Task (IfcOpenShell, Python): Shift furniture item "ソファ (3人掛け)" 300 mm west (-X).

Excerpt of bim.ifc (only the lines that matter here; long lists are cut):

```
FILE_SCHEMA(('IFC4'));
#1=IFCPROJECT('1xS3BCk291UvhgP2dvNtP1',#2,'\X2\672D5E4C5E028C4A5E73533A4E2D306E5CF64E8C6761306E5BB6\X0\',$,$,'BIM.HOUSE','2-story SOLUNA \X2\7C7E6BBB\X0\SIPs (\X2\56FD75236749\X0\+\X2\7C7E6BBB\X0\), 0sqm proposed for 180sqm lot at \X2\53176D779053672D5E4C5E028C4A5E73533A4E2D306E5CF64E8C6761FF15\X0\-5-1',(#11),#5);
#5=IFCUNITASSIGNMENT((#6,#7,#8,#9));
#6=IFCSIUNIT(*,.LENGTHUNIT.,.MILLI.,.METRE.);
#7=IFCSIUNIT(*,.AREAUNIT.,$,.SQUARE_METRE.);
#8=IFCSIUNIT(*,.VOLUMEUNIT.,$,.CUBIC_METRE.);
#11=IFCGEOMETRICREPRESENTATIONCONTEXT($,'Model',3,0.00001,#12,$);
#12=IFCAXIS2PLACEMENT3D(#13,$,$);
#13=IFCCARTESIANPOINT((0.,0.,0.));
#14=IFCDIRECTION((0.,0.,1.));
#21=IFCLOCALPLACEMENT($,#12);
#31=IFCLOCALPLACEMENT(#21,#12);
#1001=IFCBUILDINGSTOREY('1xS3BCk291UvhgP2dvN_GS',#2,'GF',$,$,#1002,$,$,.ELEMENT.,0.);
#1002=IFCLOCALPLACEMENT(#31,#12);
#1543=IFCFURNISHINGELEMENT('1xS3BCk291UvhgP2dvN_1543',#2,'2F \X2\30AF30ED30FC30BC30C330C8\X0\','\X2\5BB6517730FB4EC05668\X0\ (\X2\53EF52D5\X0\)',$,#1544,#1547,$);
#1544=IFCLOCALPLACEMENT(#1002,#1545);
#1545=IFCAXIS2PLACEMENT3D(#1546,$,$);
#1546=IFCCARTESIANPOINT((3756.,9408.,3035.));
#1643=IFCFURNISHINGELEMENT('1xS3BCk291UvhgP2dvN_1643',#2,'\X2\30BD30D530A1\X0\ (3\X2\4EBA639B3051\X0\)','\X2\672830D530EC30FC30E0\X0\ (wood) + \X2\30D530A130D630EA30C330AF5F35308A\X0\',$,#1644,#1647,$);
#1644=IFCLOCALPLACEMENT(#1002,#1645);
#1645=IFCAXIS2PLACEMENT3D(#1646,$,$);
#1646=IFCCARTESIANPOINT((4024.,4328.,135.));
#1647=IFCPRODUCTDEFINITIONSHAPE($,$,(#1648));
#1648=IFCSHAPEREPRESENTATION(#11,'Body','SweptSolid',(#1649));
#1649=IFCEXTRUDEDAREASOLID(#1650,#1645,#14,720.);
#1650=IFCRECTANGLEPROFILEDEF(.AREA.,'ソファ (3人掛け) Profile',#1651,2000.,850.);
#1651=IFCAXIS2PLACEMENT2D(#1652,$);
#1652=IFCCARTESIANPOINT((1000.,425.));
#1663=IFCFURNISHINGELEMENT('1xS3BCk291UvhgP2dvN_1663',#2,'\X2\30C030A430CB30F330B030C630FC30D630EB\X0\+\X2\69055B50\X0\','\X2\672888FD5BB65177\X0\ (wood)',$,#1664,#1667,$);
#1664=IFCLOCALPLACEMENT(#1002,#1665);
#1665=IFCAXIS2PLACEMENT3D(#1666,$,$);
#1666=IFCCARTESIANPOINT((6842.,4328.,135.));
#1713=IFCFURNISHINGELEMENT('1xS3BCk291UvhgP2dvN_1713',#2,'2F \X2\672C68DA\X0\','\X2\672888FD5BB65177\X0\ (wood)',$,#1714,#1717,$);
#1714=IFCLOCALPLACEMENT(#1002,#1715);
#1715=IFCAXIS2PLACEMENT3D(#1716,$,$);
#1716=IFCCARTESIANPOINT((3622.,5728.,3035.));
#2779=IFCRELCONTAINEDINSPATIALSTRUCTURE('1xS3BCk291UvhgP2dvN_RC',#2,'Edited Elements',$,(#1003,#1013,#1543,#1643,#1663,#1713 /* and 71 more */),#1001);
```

```python
import ifcopenshell
import ifcopenshell.api.geometry
import ifcopenshell.util.placement

model = ifcopenshell.open("bim.ifc")

item = model.by_id(1643)
matrix = ifcopenshell.util.placement.get_local_placement(item.ObjectPlacement)
matrix[0, 3] -= 300.0
ifcopenshell.api.geometry.edit_object_placement(model, product=item, matrix=matrix, is_si=False)

print(ifcopenshell.util.placement.get_local_placement(item.ObjectPlacement).round(3) + 0.0)

model.write("bim_edited.ifc")
```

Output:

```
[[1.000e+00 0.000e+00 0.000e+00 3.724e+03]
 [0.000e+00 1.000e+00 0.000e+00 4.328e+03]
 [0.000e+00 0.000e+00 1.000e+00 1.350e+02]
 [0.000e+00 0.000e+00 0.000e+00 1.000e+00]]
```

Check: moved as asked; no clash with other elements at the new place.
